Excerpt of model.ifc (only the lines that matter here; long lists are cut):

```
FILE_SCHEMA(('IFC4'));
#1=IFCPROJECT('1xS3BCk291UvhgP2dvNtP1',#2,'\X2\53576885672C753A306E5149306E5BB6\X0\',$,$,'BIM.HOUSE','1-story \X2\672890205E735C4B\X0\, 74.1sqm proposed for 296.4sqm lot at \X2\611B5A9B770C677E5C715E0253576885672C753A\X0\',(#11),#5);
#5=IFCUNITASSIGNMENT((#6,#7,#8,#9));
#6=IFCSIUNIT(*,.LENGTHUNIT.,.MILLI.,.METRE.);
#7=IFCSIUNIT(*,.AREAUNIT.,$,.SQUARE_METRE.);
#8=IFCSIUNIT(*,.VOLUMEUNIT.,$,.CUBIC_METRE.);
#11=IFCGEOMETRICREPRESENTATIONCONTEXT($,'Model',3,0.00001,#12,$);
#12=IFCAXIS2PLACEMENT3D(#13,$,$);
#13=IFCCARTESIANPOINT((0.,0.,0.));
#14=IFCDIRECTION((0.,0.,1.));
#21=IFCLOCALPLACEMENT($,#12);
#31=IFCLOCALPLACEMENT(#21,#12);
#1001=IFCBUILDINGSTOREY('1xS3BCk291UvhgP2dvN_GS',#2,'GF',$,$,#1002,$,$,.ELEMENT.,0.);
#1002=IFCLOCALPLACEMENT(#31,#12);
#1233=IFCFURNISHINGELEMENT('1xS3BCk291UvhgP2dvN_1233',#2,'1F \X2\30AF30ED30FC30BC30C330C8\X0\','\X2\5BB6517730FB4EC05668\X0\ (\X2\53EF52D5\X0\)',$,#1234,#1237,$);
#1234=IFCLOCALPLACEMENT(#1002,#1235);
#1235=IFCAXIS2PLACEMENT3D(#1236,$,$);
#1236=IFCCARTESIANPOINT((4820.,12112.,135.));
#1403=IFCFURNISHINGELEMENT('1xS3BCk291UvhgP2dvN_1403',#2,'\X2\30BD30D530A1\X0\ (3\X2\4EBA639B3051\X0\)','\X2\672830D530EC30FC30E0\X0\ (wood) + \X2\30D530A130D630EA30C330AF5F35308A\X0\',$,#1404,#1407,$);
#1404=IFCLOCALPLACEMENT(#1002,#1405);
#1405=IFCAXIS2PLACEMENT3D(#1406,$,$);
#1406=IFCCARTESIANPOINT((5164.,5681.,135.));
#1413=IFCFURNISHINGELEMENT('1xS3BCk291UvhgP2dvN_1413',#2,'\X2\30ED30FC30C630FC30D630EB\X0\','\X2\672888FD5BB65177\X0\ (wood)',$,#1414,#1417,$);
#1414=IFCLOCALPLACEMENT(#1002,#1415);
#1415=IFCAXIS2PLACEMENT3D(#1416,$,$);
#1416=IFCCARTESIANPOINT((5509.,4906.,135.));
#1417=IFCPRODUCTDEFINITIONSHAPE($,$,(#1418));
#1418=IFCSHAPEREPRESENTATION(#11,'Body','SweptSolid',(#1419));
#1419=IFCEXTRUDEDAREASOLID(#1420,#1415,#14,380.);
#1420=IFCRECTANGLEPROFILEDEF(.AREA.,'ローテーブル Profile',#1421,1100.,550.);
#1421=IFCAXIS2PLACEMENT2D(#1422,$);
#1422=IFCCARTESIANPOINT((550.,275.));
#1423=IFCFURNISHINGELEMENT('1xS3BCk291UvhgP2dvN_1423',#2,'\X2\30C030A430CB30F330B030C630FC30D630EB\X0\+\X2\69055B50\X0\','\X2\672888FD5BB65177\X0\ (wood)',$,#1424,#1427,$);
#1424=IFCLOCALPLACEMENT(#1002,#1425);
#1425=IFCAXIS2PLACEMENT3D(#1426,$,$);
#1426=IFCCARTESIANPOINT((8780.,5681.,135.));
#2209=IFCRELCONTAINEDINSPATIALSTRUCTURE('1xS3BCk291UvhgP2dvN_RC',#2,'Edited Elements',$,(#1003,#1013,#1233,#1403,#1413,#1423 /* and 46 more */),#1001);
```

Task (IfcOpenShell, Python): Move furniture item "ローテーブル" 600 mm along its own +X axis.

```python
import ifcopenshell
import ifcopenshell.api.geometry
import ifcopenshell.util.placement
import ifcopenshell.util.unit

model = ifcopenshell.open("model.ifc")
unit_scale = ifcopenshell.util.unit.calculate_unit_scale(model)

item = model.by_guid("1xS3BCk291UvhgP2dvN_1413")
matrix = ifcopenshell.util.placement.get_local_placement(item.ObjectPlacement)
matrix[:3, 3] += matrix[:3, 0] * 0.6 / unit_scale
ifcopenshell.api.geometry.edit_object_placement(model, product=item, matrix=matrix, is_si=False)

print(ifcopenshell.util.placement.get_local_placement(item.ObjectPlacement).round(3) + 0.0)

model.write("model_v2.ifc")
```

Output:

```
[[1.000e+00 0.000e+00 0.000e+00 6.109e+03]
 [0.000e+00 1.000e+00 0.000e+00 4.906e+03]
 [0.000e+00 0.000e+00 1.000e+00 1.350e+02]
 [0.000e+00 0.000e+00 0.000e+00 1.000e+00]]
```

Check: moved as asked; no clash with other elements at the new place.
